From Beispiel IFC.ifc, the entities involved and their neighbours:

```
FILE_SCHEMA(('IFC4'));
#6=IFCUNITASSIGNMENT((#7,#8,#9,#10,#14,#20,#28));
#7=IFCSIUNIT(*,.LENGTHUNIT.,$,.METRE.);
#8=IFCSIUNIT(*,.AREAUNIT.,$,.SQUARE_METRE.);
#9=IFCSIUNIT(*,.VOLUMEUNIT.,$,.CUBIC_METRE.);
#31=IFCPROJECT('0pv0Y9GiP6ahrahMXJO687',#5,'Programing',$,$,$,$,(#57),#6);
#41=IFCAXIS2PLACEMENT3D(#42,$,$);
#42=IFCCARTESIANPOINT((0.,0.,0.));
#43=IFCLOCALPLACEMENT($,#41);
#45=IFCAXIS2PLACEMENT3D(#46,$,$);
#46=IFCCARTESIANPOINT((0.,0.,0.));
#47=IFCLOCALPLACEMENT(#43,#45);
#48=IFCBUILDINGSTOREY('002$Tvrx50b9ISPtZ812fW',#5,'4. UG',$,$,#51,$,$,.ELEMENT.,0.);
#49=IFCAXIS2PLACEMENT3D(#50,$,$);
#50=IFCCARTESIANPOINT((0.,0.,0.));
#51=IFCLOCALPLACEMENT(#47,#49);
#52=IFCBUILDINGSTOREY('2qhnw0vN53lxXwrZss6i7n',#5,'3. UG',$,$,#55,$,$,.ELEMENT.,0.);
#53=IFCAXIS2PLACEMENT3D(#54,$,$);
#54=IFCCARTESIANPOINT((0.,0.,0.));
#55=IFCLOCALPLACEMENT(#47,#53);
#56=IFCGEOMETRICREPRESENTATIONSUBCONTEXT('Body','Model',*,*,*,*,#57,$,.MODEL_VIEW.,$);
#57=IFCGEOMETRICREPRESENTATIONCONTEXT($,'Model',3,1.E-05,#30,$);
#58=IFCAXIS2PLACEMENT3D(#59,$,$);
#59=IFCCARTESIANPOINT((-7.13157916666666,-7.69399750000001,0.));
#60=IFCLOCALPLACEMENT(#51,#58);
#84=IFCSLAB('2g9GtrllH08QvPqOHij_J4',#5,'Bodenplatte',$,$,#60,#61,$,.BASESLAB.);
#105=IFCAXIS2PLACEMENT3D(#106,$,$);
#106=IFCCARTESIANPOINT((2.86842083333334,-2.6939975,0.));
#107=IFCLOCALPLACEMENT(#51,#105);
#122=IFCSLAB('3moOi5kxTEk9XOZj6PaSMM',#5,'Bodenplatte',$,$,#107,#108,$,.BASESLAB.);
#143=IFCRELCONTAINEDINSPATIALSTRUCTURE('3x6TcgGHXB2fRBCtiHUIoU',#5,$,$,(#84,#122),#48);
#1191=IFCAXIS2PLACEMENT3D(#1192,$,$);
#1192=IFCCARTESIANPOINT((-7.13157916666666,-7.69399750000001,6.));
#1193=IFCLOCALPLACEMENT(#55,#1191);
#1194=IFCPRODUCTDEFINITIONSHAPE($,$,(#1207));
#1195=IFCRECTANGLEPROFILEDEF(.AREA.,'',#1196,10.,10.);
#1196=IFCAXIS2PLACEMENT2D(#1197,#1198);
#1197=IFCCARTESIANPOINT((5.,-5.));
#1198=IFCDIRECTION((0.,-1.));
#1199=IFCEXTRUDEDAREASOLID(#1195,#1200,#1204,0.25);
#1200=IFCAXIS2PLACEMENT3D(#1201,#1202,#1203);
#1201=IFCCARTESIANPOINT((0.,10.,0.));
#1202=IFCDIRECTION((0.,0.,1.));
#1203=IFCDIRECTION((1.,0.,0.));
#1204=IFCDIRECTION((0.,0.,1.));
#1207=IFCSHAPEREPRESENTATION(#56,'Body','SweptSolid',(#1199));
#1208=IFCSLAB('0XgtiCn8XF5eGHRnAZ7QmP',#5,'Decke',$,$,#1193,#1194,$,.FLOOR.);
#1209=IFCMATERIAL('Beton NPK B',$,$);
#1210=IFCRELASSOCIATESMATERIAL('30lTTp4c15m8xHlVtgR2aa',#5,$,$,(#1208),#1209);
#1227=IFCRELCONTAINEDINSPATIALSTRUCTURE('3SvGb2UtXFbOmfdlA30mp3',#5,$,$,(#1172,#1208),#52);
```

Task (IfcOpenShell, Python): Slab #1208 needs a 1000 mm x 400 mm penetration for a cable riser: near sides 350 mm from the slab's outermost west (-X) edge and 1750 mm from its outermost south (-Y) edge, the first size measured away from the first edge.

```python
import numpy as np
import ifcopenshell
import ifcopenshell.api.feature
import ifcopenshell.api.geometry
import ifcopenshell.api.root
import ifcopenshell.geom
import ifcopenshell.util.placement
import ifcopenshell.util.representation
import ifcopenshell.util.shape
import ifcopenshell.util.unit

model = ifcopenshell.open("Beispiel IFC.ifc")
unit_scale = ifcopenshell.util.unit.calculate_unit_scale(model)
settings = ifcopenshell.geom.settings()


def volume(element):
    """Net volume in cubic metres, openings subtracted."""
    shape = ifcopenshell.geom.create_shape(settings, element)
    return ifcopenshell.util.shape.get_volume(shape.geometry)


slab = model.by_guid("0XgtiCn8XF5eGHRnAZ7QmP")
before = volume(slab)

# Extent in the slab's own axes, in metres. The edges named are its -X and -Y sides.
slab_shape = ifcopenshell.geom.create_shape(settings, slab)
vertices = ifcopenshell.util.shape.get_vertices(slab_shape.geometry)
x_min, y_min, bottom = vertices.min(axis=0)
top = vertices[:, 2].max()

opening = ifcopenshell.api.root.create_entity(model, ifc_class="IfcOpeningElement", name="Cable riser opening", predefined_type="OPENING")
context = ifcopenshell.util.representation.get_context(model, "Model", "Body", "MODEL_VIEW")
width, depth = 1, 0.4
outline = [(0.0, 0.0), (width, 0.0), (width, depth), (0.0, depth), (0.0, 0.0)]
# Overshoot both faces by 50 mm so the cut is clean.
shape = ifcopenshell.api.geometry.add_slab_representation(
    model, context=context, depth=top - bottom + 0.1, polyline=outline
)
ifcopenshell.api.geometry.assign_representation(model, product=opening, representation=shape)

matrix = ifcopenshell.util.placement.get_local_placement(slab.ObjectPlacement)
matrix[:, 3] = matrix @ np.append(np.array([x_min + 0.35, y_min + 1.75, bottom - 0.05]) / unit_scale, 1.0)
ifcopenshell.api.geometry.edit_object_placement(model, product=opening, matrix=matrix, is_si=False)
ifcopenshell.api.feature.add_feature(model, feature=opening, element=slab)

after = volume(slab)

print(f"slab volume {before:.3f} -> {after:.3f} m3")

model.write("Beispiel IFC-out.ifc")
```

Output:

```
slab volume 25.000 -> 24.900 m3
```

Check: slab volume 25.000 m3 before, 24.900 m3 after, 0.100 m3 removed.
